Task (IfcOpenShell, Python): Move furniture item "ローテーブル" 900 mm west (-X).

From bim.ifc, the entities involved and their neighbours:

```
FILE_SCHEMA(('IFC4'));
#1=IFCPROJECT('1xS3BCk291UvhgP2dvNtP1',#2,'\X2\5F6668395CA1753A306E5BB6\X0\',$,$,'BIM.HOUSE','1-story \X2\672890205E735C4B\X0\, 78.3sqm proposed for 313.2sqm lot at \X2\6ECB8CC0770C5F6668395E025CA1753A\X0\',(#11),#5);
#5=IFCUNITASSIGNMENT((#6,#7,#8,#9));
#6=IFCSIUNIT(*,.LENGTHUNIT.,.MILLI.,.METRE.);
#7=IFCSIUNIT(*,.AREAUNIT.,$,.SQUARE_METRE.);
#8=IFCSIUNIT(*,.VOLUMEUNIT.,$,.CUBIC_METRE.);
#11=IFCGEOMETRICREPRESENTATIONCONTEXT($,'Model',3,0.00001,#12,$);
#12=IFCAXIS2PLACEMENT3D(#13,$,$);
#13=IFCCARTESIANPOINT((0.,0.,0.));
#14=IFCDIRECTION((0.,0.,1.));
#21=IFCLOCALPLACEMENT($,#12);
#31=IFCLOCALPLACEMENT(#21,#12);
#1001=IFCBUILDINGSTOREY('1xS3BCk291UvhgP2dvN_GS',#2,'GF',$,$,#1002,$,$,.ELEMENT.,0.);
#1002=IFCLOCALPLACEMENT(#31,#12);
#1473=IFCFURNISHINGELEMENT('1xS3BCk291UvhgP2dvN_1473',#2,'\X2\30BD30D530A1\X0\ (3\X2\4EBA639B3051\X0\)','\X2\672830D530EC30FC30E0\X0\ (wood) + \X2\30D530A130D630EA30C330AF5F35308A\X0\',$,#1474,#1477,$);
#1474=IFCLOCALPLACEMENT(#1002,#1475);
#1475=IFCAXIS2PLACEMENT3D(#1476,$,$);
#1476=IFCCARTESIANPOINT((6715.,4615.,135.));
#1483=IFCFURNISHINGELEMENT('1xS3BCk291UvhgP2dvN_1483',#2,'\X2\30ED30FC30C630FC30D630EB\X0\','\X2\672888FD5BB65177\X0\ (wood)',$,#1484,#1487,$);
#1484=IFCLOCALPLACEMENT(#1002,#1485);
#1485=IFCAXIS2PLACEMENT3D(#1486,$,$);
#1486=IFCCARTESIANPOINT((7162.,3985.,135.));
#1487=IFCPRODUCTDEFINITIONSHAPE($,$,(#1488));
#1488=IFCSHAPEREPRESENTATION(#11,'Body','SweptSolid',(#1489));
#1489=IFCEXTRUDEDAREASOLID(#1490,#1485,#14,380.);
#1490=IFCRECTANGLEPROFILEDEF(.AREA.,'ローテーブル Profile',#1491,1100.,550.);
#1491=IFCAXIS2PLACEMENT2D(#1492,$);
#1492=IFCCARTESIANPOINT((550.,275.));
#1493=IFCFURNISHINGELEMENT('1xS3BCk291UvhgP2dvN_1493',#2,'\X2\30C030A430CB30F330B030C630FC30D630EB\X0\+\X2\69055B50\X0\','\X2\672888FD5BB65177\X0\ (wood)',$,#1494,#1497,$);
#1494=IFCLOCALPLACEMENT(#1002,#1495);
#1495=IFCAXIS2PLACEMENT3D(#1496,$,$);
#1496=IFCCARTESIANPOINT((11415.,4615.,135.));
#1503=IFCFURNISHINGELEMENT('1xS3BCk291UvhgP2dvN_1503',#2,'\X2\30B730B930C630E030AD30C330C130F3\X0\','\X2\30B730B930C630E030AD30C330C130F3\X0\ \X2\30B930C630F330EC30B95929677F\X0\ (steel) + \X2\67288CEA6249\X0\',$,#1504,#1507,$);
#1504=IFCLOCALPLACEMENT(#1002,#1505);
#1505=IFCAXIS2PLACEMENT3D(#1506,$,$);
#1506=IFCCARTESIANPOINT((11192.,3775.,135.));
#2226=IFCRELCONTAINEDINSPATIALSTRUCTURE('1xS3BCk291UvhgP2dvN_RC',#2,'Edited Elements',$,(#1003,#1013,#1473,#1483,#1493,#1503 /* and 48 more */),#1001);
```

```python
import ifcopenshell
import ifcopenshell.api.geometry
import ifcopenshell.util.placement

model = ifcopenshell.open("bim.ifc")

item = model.by_guid("1xS3BCk291UvhgP2dvN_1483")
matrix = ifcopenshell.util.placement.get_local_placement(item.ObjectPlacement)
matrix[0, 3] -= 900.0
ifcopenshell.api.geometry.edit_object_placement(model, product=item, matrix=matrix, is_si=False)

print(ifcopenshell.util.placement.get_local_placement(item.ObjectPlacement).round(3) + 0.0)

model.write("bim_updated.ifc")
```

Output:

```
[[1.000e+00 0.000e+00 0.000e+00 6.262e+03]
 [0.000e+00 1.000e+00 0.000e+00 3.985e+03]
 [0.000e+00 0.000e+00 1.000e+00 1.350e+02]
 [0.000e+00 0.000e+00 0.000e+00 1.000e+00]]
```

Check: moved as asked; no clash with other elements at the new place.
